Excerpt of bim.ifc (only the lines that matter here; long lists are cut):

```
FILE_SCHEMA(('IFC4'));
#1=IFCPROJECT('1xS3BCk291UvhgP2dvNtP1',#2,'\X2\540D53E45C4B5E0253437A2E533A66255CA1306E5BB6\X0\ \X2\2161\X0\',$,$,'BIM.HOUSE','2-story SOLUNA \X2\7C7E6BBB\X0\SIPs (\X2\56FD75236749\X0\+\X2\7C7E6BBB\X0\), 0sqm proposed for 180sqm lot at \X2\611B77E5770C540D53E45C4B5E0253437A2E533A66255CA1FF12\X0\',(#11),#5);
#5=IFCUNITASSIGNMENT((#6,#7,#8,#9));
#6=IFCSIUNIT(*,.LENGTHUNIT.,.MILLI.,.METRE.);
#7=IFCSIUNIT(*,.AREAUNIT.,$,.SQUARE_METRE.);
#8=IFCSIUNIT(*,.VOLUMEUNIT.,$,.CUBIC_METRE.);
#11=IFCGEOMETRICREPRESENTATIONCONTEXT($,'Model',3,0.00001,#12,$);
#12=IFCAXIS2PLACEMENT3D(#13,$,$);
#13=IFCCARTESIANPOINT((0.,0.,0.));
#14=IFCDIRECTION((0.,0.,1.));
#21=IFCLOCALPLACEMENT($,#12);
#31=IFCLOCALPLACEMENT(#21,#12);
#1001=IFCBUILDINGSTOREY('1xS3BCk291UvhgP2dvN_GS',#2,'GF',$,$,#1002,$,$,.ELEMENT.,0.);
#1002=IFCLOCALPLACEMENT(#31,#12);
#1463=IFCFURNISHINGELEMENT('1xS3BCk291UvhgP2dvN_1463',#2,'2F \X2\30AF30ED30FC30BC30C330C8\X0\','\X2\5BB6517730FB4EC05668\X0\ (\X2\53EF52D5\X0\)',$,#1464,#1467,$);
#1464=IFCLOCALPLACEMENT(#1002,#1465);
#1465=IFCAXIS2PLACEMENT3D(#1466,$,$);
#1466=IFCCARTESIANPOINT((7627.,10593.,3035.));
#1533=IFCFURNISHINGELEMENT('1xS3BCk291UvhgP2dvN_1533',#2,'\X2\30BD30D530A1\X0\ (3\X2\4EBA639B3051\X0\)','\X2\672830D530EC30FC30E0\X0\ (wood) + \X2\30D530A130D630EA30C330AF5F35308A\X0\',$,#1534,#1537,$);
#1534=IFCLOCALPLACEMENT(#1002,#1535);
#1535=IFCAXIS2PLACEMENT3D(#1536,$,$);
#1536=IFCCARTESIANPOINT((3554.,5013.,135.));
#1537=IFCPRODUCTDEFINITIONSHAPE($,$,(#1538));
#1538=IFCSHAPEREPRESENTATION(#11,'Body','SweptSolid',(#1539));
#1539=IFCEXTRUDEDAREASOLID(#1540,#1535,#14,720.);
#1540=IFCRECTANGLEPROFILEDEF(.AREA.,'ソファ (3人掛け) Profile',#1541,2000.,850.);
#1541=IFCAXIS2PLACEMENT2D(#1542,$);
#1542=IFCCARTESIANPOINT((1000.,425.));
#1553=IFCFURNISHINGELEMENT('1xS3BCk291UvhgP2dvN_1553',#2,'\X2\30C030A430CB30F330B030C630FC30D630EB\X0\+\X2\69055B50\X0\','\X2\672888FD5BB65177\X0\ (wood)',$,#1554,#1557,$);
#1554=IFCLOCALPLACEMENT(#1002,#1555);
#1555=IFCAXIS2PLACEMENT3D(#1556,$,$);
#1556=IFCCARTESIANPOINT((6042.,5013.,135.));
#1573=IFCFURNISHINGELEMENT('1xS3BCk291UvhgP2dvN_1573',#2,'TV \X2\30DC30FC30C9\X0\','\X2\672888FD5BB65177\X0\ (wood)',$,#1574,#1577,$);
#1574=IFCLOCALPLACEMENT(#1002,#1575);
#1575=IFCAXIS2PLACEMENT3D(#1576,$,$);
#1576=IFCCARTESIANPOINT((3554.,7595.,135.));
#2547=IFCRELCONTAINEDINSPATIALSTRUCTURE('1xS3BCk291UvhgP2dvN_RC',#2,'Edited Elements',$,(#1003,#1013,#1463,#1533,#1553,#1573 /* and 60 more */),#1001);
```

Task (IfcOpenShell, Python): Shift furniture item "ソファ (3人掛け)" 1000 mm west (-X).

```python
import ifcopenshell
import ifcopenshell.api.geometry
import ifcopenshell.util.placement
import ifcopenshell.util.unit

model = ifcopenshell.open("bim.ifc")
unit_scale = ifcopenshell.util.unit.calculate_unit_scale(model)

item = model.by_guid("1xS3BCk291UvhgP2dvN_1533")
matrix = ifcopenshell.util.placement.get_local_placement(item.ObjectPlacement)
matrix[0, 3] -= 1 / unit_scale
ifcopenshell.api.geometry.edit_object_placement(model, product=item, matrix=matrix, is_si=False)

print(ifcopenshell.util.placement.get_local_placement(item.ObjectPlacement).round(3) + 0.0)

model.write("bim_rev.ifc")
```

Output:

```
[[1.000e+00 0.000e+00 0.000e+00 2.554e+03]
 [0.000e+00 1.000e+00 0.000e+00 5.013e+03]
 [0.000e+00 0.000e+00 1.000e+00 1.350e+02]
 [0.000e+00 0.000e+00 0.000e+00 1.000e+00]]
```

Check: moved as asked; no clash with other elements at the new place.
